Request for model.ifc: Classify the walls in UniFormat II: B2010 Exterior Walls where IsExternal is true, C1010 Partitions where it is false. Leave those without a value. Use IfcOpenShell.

First a look at what the model holds.

```python
import ifcopenshell
import ifcopenshell.util.element

model = ifcopenshell.open("model.ifc")
print(model.schema)
print("classifications:", [c.Name for c in model.by_type("IfcClassification")])
values = [ifcopenshell.util.element.get_pset(e, "Pset_WallCommon", "IsExternal") for e in model.by_type("IfcWall")]
for value in (True, False, None):
    print("IsExternal", value, values.count(value))
```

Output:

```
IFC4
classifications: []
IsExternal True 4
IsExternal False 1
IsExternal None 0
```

```python
import ifcopenshell
import ifcopenshell.api.classification
import ifcopenshell.util.element

model = ifcopenshell.open("model.ifc")

system = ifcopenshell.api.classification.add_classification(model, classification="UniFormat II")

walls = model.by_type("IfcWall")
external = {e: ifcopenshell.util.element.get_pset(e, "Pset_WallCommon", "IsExternal") for e in walls}
for flag, code, name in ((True, "B2010", "Exterior Walls"), (False, "C1010", "Partitions")):
    products = [e for e in walls if external[e] is flag]
    ifcopenshell.api.classification.add_reference(
        model, products=products, classification=system, identification=code, name=name
    )
    print(code, len(products))

model.write("model_updated.ifc")
```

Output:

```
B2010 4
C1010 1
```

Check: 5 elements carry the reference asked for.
